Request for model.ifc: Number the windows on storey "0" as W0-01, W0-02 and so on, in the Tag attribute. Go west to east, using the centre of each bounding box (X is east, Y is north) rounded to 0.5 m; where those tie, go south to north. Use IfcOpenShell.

First a look at what the model holds.

```python
import ifcopenshell
import ifcopenshell.util.element
import ifcopenshell.util.placement

model = ifcopenshell.open("model.ifc")
print(model.schema)
storey = next(s for s in model.by_type("IfcBuildingStorey") if s.Name == "0")
windows = [e for e in ifcopenshell.util.element.get_decomposition(storey) if e.is_a("IfcWindow")]
for e in sorted(windows, key=lambda e: e.id()):
    origin = ifcopenshell.util.placement.get_local_placement(e.ObjectPlacement)[:3, 3]
    print(e.id(), e.Tag, e.Name, origin.round(2) + 0.0, sep=" | ")
```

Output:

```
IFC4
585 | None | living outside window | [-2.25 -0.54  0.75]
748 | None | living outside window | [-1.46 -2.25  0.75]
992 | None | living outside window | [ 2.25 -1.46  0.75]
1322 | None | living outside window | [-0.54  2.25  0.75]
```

```python
import ifcopenshell
import ifcopenshell.geom
import ifcopenshell.util.element
import ifcopenshell.util.shape

model = ifcopenshell.open("model.ifc")
settings = ifcopenshell.geom.settings()
settings.set("use-world-coords", True)


def centre(element):
    shape = ifcopenshell.geom.create_shape(settings, element)
    return ifcopenshell.util.shape.get_bbox_centroid(shape.geometry)


storey = next(s for s in model.by_type("IfcBuildingStorey") if s.Name == "0")
windows = [e for e in ifcopenshell.util.element.get_decomposition(storey) if e.is_a("IfcWindow")]

# Insertion points can sit at a corner or the storey origin, so sort by the geometry (in metres).
centres = {e: centre(e) for e in windows}
windows.sort(key=lambda e: (round(centres[e][0] / 0.5), centres[e][1]))

for i, e in enumerate(windows, start=1):
    number = f"W0-{i:02d}"
    e.Tag = number
    print(e.id(), number)

model.write("model_v2.ifc")
```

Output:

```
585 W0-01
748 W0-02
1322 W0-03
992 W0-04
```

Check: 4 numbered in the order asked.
